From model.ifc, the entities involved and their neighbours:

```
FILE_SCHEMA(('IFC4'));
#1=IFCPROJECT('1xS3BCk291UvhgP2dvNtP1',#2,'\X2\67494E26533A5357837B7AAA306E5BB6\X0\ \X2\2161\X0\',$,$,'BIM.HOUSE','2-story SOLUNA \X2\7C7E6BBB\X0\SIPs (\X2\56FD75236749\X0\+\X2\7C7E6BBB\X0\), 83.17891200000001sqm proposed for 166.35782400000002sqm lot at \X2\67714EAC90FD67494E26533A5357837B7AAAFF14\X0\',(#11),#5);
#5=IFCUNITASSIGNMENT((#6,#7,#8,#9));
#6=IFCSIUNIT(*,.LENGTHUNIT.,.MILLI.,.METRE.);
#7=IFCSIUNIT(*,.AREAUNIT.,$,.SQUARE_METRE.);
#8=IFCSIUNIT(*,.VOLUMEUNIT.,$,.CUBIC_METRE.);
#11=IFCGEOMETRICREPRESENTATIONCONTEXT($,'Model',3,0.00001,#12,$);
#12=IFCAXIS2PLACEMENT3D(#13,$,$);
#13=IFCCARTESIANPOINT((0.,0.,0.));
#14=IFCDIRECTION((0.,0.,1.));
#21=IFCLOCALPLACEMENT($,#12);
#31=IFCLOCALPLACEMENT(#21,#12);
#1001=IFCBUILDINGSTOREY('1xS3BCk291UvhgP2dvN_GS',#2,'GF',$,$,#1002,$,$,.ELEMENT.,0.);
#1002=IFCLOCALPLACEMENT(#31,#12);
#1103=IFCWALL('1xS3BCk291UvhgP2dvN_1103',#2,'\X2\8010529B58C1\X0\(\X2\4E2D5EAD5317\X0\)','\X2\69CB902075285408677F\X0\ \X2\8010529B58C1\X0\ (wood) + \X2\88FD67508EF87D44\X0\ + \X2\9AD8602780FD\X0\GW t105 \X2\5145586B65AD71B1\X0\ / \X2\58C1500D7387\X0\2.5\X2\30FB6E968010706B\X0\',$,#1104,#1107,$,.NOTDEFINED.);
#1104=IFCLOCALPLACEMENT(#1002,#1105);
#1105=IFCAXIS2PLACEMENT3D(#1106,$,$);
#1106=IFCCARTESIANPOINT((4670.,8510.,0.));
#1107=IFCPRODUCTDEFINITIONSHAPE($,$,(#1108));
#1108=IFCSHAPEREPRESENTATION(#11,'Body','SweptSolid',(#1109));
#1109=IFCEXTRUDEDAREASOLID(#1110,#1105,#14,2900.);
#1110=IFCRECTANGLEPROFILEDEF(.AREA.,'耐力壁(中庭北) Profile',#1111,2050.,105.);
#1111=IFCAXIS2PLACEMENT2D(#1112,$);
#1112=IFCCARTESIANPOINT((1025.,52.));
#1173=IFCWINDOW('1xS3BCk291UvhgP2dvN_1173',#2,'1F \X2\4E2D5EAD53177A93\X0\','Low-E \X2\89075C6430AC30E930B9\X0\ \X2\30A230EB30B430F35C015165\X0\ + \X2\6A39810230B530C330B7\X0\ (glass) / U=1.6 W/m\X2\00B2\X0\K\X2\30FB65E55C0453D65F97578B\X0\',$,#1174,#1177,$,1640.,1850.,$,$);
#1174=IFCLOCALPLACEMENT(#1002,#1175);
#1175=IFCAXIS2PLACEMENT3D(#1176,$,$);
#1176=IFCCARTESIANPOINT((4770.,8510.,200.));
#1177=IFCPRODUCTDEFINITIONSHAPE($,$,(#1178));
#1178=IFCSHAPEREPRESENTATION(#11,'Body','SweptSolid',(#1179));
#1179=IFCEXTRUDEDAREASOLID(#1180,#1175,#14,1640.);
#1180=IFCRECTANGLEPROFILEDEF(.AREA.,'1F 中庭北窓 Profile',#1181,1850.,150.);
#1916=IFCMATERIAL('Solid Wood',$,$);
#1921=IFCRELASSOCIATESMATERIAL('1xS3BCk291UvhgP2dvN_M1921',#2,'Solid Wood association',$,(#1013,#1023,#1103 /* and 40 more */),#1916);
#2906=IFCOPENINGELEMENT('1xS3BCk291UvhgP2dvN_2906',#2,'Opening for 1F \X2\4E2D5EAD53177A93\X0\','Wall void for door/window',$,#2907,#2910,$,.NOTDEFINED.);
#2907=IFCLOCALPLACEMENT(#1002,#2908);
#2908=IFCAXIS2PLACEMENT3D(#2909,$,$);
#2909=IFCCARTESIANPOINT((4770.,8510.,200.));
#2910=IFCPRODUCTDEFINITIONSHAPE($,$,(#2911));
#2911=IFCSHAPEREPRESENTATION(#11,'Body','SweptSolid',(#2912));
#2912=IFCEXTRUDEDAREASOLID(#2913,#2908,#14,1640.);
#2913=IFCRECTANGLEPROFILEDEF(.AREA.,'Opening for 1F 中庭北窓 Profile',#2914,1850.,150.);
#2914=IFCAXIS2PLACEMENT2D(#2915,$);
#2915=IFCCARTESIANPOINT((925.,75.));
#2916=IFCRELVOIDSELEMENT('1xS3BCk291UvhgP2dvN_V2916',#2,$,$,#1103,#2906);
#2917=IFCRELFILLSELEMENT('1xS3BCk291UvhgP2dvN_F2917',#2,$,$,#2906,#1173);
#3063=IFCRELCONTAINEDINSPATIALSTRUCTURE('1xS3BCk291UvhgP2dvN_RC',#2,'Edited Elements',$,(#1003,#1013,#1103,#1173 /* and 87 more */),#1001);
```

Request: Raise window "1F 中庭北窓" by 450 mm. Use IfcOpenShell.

```python
import numpy as np
import ifcopenshell
import ifcopenshell.api.geometry
import ifcopenshell.util.placement
import ifcopenshell.util.unit

model = ifcopenshell.open("model.ifc")
unit_scale = ifcopenshell.util.unit.calculate_unit_scale(model)

window = model.by_guid("1xS3BCk291UvhgP2dvN_1173")
opening = window.FillsVoids[0].RelatingOpeningElement
dz = 0.45 / unit_scale

shift = np.array([0.0, 0.0, dz])
# The window is not placed relative to its opening, so move both.
for product in (opening, window):
    matrix = ifcopenshell.util.placement.get_local_placement(product.ObjectPlacement)
    matrix[:3, 3] += shift
    ifcopenshell.api.geometry.edit_object_placement(model, product=product, matrix=matrix, is_si=False)

print(f"moved by {dz * unit_scale:+.3f} m")

model.write("model_v2.ifc")
```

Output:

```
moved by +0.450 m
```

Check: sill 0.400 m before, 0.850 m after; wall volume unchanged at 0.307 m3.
